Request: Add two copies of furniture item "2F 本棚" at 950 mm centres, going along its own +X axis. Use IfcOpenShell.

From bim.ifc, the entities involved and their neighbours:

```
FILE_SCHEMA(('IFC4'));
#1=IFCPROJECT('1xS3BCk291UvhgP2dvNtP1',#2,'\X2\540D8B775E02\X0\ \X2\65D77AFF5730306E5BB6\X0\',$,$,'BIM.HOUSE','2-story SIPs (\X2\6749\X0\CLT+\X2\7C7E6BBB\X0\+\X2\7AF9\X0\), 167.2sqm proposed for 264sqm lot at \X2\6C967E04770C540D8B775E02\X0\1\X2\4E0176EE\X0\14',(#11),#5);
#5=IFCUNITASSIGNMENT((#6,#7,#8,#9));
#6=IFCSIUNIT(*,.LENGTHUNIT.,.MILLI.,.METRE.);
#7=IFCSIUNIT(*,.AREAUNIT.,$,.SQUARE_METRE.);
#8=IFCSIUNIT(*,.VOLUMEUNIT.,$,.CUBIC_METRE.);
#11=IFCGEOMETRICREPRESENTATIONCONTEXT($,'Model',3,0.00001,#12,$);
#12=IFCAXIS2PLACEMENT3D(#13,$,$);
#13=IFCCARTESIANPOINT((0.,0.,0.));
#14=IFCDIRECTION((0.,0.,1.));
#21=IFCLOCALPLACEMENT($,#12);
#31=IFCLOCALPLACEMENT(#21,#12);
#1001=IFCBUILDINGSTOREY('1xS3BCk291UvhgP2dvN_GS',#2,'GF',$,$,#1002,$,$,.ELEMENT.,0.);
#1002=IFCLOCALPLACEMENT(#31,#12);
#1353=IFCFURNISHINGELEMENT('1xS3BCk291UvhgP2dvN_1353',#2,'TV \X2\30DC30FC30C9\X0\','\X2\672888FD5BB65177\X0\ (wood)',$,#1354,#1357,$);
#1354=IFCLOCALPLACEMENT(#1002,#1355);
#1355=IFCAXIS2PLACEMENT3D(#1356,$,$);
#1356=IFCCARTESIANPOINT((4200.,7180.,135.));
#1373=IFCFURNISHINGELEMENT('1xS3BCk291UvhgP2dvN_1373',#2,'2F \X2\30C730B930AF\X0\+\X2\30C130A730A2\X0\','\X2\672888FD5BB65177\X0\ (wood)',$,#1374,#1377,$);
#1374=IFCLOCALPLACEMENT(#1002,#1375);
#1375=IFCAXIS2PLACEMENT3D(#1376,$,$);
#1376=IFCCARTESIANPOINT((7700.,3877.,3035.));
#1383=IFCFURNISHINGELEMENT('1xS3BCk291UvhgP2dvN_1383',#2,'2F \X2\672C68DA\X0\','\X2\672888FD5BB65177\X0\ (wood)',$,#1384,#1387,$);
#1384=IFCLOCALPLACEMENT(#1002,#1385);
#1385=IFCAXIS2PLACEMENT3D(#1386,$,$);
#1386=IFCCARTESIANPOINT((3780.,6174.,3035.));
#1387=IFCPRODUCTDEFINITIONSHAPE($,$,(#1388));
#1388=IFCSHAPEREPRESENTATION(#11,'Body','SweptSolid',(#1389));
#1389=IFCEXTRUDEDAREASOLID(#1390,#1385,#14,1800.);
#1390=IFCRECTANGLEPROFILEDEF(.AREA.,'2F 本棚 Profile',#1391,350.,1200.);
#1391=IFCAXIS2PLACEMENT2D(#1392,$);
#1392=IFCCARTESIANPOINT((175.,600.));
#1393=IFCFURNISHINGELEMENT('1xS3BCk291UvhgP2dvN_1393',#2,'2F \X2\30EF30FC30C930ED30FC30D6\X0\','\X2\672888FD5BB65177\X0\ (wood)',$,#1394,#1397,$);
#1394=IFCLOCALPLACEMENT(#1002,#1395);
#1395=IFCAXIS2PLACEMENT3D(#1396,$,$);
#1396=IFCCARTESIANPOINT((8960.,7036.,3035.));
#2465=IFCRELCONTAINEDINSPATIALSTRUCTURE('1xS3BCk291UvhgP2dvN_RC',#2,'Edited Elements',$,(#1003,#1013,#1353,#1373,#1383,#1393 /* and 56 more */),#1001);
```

```python
import ifcopenshell
import ifcopenshell.api.geometry
import ifcopenshell.api.root
import ifcopenshell.util.element
import ifcopenshell.util.placement

model = ifcopenshell.open("bim.ifc")


def reuse_history(source, copy):
    """copy_class also copies each property set's owner history, people and application; keep the originals."""
    for rel in copy.IsDefinedBy:
        if rel.is_a("IfcRelDefinesByProperties") and (history := rel.RelatingPropertyDefinition.OwnerHistory):
            rel.RelatingPropertyDefinition.OwnerHistory = source.OwnerHistory
            ifcopenshell.util.element.remove_deep2(model, history)


source = model.by_id(1383)
base = ifcopenshell.util.placement.get_local_placement(source.ObjectPlacement)
step = base[:3, 0] * 950.0

for i in range(1, 3):
    copy = ifcopenshell.api.root.copy_class(model, product=source)
    copy.Representation = ifcopenshell.util.element.copy_deep(
        model, source.Representation, exclude=["IfcGeometricRepresentationContext", "IfcRepresentationMap"]
    )
    reuse_history(source, copy)
    matrix = base.copy()
    matrix[:3, 3] += i * step
    print("added at", matrix[:3, 3].round(3) + 0.0)
    ifcopenshell.api.geometry.edit_object_placement(model, product=copy, matrix=matrix, is_si=False)

model.write("bim-out.ifc")
```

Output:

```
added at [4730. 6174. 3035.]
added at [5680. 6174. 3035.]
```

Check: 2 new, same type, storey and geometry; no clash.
